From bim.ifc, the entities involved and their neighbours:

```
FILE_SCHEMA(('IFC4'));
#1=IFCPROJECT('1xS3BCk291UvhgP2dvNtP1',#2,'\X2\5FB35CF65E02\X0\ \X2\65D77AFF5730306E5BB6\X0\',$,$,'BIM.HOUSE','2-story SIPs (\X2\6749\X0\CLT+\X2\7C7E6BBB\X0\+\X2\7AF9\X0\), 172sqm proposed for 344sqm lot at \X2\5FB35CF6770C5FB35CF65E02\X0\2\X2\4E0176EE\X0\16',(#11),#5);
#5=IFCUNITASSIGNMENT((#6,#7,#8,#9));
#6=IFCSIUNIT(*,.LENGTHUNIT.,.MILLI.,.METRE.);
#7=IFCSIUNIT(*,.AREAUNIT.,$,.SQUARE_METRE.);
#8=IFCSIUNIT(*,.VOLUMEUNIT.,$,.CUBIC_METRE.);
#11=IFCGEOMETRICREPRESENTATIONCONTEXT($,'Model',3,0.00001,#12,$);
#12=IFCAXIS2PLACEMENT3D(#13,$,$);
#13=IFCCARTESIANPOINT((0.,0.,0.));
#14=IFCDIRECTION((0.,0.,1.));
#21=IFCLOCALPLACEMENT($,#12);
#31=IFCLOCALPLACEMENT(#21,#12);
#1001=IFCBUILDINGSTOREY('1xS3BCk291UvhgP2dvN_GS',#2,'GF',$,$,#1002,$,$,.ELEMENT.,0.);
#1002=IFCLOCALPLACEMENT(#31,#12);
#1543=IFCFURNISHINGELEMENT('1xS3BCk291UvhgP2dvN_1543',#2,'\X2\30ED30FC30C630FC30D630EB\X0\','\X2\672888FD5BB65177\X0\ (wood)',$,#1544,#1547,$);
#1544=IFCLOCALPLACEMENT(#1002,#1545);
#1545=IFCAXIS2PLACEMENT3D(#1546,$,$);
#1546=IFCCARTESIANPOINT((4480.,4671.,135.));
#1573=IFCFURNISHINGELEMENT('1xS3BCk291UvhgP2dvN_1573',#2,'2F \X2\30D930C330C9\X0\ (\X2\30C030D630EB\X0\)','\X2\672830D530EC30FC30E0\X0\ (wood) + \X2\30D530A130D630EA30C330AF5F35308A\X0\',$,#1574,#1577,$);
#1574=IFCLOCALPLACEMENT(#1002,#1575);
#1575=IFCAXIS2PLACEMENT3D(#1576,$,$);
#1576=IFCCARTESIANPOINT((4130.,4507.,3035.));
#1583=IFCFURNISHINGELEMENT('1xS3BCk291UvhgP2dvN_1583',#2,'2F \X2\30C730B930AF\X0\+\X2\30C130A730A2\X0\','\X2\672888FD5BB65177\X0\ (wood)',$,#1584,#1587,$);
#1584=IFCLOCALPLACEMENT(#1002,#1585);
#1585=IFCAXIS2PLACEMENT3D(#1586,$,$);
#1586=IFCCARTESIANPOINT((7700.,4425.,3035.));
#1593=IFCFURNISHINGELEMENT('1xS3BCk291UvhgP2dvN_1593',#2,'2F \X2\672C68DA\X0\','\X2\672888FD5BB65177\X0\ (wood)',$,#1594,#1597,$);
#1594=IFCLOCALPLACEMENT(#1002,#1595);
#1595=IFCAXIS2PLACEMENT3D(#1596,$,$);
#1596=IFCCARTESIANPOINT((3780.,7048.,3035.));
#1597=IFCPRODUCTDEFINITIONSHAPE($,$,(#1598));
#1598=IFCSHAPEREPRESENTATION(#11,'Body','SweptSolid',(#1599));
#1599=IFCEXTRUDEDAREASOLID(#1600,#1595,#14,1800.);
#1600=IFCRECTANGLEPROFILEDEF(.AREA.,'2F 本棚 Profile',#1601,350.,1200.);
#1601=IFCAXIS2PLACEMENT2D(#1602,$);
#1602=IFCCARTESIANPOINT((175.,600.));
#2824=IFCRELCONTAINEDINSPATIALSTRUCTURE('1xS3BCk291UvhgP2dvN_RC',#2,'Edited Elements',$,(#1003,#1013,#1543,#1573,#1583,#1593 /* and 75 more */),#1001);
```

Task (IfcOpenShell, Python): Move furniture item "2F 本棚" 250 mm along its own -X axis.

```python
import ifcopenshell
import ifcopenshell.api.geometry
import ifcopenshell.util.placement
import ifcopenshell.util.unit

model = ifcopenshell.open("bim.ifc")
unit_scale = ifcopenshell.util.unit.calculate_unit_scale(model)

item = model.by_guid("1xS3BCk291UvhgP2dvN_1593")
matrix = ifcopenshell.util.placement.get_local_placement(item.ObjectPlacement)
matrix[:3, 3] -= matrix[:3, 0] * 0.25 / unit_scale
ifcopenshell.api.geometry.edit_object_placement(model, product=item, matrix=matrix, is_si=False)

print(ifcopenshell.util.placement.get_local_placement(item.ObjectPlacement).round(3) + 0.0)

model.write("bim_rev.ifc")
```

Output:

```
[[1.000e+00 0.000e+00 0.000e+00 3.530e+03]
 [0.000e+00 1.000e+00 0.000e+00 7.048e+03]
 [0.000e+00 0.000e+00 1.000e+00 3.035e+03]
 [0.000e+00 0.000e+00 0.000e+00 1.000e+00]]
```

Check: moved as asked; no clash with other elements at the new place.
